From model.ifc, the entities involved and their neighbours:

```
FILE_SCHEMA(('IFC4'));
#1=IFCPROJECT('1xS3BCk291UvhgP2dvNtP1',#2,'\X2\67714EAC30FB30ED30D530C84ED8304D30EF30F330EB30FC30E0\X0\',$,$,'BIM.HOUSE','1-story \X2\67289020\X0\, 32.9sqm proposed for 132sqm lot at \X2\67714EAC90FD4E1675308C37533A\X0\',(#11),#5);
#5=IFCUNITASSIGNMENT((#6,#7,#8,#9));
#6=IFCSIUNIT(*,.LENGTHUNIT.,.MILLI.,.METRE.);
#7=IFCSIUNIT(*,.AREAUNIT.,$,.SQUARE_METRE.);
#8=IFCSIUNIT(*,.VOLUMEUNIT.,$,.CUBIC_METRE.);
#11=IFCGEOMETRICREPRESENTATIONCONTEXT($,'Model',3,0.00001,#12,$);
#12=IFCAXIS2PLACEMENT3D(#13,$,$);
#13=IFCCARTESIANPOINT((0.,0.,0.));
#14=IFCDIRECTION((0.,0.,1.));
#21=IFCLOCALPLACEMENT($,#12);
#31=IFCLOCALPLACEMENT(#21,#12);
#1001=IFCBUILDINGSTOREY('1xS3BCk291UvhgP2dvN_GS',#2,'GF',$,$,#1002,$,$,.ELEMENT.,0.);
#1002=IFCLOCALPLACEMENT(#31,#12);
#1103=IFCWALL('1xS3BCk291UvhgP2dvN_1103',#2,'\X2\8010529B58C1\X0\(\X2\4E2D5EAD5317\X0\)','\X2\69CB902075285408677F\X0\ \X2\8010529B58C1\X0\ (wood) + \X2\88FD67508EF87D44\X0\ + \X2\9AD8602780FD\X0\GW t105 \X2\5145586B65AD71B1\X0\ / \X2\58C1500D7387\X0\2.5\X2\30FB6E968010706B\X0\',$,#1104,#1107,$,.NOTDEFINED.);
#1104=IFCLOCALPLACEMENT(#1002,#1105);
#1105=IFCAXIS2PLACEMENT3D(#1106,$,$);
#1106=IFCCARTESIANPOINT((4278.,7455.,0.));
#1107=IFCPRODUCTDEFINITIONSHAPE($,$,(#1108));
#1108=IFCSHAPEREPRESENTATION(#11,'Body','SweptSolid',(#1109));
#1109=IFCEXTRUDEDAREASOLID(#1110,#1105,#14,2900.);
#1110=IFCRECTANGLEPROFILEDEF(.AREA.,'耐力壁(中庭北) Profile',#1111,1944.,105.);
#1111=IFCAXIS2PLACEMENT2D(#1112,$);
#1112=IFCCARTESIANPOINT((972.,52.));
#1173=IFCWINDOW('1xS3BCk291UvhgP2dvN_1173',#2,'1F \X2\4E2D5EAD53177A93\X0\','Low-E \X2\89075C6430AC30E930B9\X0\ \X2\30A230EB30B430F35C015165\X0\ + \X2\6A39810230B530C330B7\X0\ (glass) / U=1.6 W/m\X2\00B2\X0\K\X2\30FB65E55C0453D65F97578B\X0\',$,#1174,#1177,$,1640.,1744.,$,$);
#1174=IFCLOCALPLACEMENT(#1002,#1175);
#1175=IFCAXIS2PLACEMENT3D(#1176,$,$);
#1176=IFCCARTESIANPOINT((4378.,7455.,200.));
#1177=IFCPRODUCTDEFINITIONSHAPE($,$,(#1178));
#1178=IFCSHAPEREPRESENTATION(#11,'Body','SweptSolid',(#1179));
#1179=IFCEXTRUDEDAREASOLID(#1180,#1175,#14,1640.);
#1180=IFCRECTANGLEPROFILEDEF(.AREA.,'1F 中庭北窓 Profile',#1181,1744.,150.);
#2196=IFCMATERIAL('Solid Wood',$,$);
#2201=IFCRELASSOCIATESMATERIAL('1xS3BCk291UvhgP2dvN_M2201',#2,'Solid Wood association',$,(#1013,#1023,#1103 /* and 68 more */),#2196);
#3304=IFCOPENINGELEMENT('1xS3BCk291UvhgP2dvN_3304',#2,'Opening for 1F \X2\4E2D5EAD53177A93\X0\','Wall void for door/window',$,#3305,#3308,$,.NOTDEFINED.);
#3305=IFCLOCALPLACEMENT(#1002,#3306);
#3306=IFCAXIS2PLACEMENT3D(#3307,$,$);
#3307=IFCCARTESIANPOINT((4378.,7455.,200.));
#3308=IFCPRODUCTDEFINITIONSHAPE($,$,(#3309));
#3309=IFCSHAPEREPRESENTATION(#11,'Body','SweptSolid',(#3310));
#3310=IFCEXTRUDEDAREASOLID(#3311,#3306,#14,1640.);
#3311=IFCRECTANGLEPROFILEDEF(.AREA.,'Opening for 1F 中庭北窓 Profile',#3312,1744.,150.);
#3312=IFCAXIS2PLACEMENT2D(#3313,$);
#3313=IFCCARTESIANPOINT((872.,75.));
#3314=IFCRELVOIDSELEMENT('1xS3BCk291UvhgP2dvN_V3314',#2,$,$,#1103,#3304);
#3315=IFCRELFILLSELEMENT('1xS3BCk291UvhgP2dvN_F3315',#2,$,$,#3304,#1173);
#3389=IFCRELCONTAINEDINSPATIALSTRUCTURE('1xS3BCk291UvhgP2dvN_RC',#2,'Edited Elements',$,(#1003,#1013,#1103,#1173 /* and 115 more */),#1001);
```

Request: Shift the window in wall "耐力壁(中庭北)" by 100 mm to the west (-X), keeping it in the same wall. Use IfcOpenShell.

```python
import ifcopenshell
import ifcopenshell.api.geometry
import ifcopenshell.util.placement
import ifcopenshell.util.unit

model = ifcopenshell.open("model.ifc")
unit_scale = ifcopenshell.util.unit.calculate_unit_scale(model)

window = model.by_guid("1xS3BCk291UvhgP2dvN_1173")
opening = window.FillsVoids[0].RelatingOpeningElement
wall = opening.VoidsElements[0].RelatingBuildingElement

wall_matrix = ifcopenshell.util.placement.get_local_placement(wall.ObjectPlacement)
shift = wall_matrix[:3, 0] * -0.1 / unit_scale
before = ifcopenshell.util.placement.get_local_placement(window.ObjectPlacement)[:3, 3].copy()

# The window is not placed relative to its opening, so move both.
for product in (opening, window):
    matrix = ifcopenshell.util.placement.get_local_placement(product.ObjectPlacement)
    matrix[:3, 3] += shift
    ifcopenshell.api.geometry.edit_object_placement(model, product=product, matrix=matrix, is_si=False)

after = ifcopenshell.util.placement.get_local_placement(window.ObjectPlacement)[:3, 3]
print("window moved by", (after - before).round(3) + 0.0)

model.write("model_v2.ifc")
```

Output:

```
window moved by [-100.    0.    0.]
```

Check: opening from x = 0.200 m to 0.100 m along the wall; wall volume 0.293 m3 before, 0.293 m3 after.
